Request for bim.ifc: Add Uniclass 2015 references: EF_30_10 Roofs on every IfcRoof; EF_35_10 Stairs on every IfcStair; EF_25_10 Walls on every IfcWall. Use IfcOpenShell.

First a look at what the model holds.

```python
import ifcopenshell

model = ifcopenshell.open("bim.ifc")
print(model.schema)
print("classifications:", [c.Name for c in model.by_type("IfcClassification")])
for ifc_class in ("IfcDoor", "IfcRoof", "IfcStair", "IfcWall", "IfcWindow"):
    print(ifc_class, len(model.by_type(ifc_class)))
```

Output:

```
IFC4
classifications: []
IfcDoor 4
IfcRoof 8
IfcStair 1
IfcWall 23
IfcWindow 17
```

```python
import ifcopenshell
import ifcopenshell.api.classification

model = ifcopenshell.open("bim.ifc")

system = ifcopenshell.api.classification.add_classification(model, classification="Uniclass 2015")

codes = {
    "IfcRoof": ("EF_30_10", "Roofs"),
    "IfcStair": ("EF_35_10", "Stairs"),
    "IfcWall": ("EF_25_10", "Walls"),
}
for ifc_class, (code, name) in codes.items():
    products = model.by_type(ifc_class)
    ifcopenshell.api.classification.add_reference(
        model, products=products, classification=system, identification=code, name=name
    )
    print(code, len(products))

model.write("bim-out.ifc")
```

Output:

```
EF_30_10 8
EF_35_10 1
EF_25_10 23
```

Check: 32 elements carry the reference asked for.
